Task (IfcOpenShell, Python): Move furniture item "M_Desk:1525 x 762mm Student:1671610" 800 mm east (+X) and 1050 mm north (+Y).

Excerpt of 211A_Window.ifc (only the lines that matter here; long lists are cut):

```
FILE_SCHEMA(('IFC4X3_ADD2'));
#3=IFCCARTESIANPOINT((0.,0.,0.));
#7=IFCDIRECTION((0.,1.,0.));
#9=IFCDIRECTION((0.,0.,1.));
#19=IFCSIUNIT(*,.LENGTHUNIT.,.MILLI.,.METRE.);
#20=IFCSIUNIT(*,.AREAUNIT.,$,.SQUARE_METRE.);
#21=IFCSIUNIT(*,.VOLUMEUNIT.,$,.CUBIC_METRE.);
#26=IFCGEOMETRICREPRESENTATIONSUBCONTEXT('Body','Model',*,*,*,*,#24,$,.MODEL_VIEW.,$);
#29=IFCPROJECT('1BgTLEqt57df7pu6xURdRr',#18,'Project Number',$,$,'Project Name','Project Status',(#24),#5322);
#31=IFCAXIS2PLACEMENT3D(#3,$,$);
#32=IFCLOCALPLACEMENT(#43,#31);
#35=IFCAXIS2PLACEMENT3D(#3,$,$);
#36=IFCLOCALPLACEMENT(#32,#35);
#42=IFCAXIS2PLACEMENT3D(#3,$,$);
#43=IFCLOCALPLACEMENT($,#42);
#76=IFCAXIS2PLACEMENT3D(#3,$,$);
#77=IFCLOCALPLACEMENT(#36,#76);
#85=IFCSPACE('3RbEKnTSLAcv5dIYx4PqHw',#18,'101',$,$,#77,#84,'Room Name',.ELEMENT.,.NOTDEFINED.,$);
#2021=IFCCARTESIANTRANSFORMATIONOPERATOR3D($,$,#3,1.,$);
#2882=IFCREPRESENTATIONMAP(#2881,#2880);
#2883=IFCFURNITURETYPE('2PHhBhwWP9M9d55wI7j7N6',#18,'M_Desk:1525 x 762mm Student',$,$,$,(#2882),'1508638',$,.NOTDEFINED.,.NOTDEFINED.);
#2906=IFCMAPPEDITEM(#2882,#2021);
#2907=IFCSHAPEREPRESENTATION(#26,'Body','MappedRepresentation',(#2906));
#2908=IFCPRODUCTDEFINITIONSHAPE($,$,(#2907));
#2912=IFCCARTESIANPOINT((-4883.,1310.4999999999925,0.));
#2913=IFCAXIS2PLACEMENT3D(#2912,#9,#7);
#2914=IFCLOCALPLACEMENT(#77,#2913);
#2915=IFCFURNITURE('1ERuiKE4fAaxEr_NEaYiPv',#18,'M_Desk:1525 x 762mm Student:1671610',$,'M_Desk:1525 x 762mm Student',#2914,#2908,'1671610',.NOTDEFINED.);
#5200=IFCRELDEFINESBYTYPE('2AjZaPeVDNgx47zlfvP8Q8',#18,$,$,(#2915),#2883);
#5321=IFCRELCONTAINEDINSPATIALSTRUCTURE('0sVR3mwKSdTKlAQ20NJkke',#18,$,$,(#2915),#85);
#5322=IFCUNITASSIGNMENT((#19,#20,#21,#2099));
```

```python
import ifcopenshell
import ifcopenshell.api.geometry
import ifcopenshell.util.placement
import ifcopenshell.util.unit

model = ifcopenshell.open("211A_Window.ifc")
unit_scale = ifcopenshell.util.unit.calculate_unit_scale(model)

item = model.by_guid("1ERuiKE4fAaxEr_NEaYiPv")
matrix = ifcopenshell.util.placement.get_local_placement(item.ObjectPlacement)
matrix[0, 3] += 0.8 / unit_scale
matrix[1, 3] += 1.05 / unit_scale
ifcopenshell.api.geometry.edit_object_placement(model, product=item, matrix=matrix, is_si=False)

print(ifcopenshell.util.placement.get_local_placement(item.ObjectPlacement).round(3) + 0.0)

model.write("211A_Window_v2.ifc")
```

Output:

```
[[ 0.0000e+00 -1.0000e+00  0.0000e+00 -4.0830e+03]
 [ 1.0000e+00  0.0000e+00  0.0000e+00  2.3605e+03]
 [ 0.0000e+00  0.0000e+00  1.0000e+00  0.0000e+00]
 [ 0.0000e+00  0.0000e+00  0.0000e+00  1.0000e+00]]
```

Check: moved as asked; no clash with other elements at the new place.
